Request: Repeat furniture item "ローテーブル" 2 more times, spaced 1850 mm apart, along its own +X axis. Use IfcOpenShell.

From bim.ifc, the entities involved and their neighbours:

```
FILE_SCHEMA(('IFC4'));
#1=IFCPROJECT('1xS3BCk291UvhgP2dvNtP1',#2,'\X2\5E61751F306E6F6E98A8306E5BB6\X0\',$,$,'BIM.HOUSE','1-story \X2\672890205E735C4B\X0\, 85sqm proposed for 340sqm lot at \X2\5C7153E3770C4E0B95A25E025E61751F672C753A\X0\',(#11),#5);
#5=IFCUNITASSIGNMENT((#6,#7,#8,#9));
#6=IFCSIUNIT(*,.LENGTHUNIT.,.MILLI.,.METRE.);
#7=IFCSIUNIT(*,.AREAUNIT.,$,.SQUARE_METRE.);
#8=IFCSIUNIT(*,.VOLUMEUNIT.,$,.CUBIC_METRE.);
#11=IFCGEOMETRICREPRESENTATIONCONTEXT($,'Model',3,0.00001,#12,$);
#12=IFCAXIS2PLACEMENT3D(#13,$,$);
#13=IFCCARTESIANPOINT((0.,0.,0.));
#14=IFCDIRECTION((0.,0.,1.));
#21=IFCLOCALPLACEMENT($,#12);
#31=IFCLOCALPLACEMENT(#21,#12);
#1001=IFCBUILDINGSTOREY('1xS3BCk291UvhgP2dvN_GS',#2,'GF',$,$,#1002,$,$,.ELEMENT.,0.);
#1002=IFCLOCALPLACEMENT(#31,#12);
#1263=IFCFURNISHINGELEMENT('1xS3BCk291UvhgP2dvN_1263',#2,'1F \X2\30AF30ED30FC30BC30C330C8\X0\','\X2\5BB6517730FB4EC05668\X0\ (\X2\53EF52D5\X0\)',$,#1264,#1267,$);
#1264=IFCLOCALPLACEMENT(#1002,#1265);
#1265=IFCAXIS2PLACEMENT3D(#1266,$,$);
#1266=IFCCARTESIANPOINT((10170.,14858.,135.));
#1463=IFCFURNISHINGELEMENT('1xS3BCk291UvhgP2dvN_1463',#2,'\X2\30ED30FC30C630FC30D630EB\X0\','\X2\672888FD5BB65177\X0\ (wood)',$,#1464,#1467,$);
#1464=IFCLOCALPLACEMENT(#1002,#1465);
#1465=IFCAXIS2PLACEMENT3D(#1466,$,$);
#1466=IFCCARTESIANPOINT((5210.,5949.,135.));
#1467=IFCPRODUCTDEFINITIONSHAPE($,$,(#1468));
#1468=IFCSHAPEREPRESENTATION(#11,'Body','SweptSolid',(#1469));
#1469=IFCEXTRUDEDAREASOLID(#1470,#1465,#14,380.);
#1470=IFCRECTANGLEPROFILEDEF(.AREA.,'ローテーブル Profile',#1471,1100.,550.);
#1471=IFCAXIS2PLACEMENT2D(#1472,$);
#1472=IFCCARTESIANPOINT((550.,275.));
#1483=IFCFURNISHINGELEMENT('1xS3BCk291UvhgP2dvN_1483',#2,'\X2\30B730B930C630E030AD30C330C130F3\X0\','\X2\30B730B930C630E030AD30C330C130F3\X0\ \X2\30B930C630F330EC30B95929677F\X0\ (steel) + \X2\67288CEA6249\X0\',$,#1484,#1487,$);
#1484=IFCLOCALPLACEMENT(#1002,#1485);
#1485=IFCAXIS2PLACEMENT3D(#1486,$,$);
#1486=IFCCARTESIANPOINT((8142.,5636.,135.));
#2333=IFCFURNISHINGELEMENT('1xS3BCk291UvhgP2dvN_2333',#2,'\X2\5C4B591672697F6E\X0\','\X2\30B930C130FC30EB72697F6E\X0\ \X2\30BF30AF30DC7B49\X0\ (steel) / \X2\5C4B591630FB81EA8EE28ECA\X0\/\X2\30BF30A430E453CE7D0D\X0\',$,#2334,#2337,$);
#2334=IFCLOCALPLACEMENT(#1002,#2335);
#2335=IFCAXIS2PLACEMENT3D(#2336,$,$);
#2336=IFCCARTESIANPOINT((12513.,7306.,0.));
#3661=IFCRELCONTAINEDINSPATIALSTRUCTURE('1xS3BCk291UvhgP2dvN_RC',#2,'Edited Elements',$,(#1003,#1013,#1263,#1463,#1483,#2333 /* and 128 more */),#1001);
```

```python
import ifcopenshell
import ifcopenshell.api.geometry
import ifcopenshell.api.root
import ifcopenshell.util.element
import ifcopenshell.util.placement

model = ifcopenshell.open("bim.ifc")


def reuse_history(source, copy):
    """copy_class also copies each property set's owner history, people and application; keep the originals."""
    for rel in copy.IsDefinedBy:
        if rel.is_a("IfcRelDefinesByProperties") and (history := rel.RelatingPropertyDefinition.OwnerHistory):
            rel.RelatingPropertyDefinition.OwnerHistory = source.OwnerHistory
            ifcopenshell.util.element.remove_deep2(model, history)


source = model.by_id(1463)
base = ifcopenshell.util.placement.get_local_placement(source.ObjectPlacement)
step = base[:3, 0] * 1850.0

for i in range(1, 3):
    copy = ifcopenshell.api.root.copy_class(model, product=source)
    copy.Representation = ifcopenshell.util.element.copy_deep(
        model, source.Representation, exclude=["IfcGeometricRepresentationContext", "IfcRepresentationMap"]
    )
    reuse_history(source, copy)
    matrix = base.copy()
    matrix[:3, 3] += i * step
    print("added at", matrix[:3, 3].round(3) + 0.0)
    ifcopenshell.api.geometry.edit_object_placement(model, product=copy, matrix=matrix, is_si=False)

model.write("bim_edited.ifc")
```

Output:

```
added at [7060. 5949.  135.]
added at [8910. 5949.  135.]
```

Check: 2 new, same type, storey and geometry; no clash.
